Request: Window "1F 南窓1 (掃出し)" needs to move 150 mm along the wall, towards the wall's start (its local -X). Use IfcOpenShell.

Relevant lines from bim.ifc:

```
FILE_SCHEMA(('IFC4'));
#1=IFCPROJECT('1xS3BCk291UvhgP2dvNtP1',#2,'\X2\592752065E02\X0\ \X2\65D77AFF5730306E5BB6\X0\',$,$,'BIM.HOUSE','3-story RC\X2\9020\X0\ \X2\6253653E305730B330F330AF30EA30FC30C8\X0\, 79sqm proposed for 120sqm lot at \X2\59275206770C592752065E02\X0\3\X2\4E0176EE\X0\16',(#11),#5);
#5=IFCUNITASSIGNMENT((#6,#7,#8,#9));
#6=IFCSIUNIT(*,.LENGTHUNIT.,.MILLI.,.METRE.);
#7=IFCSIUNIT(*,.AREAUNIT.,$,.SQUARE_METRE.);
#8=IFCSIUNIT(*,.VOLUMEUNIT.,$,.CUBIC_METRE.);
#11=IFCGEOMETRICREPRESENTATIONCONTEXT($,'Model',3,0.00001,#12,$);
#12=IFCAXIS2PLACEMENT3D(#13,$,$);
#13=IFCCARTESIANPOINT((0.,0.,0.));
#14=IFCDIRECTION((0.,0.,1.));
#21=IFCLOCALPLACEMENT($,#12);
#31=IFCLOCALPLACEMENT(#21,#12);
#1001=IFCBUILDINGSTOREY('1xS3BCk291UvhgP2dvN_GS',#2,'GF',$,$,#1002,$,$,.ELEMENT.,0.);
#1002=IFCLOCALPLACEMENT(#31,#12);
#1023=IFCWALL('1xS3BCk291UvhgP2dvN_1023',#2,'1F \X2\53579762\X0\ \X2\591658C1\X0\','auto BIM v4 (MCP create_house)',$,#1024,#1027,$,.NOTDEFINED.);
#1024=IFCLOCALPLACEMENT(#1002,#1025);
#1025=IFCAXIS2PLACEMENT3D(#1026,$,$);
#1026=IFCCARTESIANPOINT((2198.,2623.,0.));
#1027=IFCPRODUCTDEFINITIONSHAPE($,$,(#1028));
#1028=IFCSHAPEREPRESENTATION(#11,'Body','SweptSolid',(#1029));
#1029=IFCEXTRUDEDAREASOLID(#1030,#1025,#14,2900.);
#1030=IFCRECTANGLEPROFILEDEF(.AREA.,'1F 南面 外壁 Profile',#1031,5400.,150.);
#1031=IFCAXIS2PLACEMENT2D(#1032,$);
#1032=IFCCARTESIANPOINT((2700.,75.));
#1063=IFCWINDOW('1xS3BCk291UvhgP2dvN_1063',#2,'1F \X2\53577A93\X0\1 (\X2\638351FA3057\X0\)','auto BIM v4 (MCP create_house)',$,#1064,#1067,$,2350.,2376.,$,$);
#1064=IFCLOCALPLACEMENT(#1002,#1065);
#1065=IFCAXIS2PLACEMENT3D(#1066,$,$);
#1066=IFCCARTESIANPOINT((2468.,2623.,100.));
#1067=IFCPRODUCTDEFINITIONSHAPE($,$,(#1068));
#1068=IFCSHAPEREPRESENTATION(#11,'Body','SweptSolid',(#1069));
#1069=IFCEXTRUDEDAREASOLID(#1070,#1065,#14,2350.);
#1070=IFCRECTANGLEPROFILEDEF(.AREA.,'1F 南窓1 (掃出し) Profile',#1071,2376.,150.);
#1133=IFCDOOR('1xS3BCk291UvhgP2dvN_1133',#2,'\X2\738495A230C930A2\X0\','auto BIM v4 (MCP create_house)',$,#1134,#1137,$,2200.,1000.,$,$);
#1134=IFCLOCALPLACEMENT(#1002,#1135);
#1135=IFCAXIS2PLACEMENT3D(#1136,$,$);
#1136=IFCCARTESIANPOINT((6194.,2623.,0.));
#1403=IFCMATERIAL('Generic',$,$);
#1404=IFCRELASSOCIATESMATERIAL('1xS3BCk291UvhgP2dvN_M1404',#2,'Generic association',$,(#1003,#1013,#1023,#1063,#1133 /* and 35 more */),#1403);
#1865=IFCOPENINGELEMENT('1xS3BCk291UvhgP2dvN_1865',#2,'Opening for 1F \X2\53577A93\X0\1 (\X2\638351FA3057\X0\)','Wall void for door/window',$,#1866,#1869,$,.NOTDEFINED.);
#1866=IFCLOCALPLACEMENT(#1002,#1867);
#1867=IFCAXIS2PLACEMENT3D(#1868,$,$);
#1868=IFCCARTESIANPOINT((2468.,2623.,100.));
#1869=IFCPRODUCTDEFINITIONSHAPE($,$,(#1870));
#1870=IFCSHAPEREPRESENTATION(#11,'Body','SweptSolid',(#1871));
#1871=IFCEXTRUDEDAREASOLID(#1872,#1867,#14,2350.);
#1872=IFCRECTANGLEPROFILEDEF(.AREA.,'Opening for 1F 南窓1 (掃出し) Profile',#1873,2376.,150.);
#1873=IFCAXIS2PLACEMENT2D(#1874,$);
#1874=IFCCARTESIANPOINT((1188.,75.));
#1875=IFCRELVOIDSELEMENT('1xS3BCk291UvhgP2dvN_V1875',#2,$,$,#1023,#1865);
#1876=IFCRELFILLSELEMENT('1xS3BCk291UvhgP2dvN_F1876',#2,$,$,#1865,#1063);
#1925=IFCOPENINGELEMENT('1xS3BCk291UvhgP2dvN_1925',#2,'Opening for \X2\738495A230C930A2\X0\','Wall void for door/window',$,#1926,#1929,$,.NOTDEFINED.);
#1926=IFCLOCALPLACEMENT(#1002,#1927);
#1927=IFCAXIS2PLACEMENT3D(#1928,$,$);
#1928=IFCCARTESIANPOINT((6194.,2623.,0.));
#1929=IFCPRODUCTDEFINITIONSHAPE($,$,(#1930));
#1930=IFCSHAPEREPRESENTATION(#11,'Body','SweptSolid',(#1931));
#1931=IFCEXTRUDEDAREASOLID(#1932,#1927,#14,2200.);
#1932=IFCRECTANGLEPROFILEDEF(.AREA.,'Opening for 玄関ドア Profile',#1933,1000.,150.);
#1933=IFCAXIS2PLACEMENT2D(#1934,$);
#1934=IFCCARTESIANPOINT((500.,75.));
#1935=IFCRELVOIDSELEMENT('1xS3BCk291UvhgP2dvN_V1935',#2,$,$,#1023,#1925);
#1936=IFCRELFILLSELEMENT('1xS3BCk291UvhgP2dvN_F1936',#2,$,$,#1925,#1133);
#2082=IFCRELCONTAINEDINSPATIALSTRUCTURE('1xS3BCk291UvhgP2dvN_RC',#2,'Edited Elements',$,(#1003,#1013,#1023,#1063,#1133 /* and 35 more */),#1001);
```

```python
import ifcopenshell
import ifcopenshell.api.geometry
import ifcopenshell.util.placement
import ifcopenshell.util.unit

model = ifcopenshell.open("bim.ifc")
unit_scale = ifcopenshell.util.unit.calculate_unit_scale(model)

window = model.by_id(1063)
opening = window.FillsVoids[0].RelatingOpeningElement
wall = opening.VoidsElements[0].RelatingBuildingElement

wall_matrix = ifcopenshell.util.placement.get_local_placement(wall.ObjectPlacement)
shift = wall_matrix[:3, 0] * -0.15 / unit_scale
before = ifcopenshell.util.placement.get_local_placement(window.ObjectPlacement)[:3, 3].copy()

# The window is not placed relative to its opening, so move both.
for product in (opening, window):
    matrix = ifcopenshell.util.placement.get_local_placement(product.ObjectPlacement)
    matrix[:3, 3] += shift
    ifcopenshell.api.geometry.edit_object_placement(model, product=product, matrix=matrix, is_si=False)

after = ifcopenshell.util.placement.get_local_placement(window.ObjectPlacement)[:3, 3]
print("window moved by", (after - before).round(3) + 0.0)

model.write("bim_rev.ifc")
```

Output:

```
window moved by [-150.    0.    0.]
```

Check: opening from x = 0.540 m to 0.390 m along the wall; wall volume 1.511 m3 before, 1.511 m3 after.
